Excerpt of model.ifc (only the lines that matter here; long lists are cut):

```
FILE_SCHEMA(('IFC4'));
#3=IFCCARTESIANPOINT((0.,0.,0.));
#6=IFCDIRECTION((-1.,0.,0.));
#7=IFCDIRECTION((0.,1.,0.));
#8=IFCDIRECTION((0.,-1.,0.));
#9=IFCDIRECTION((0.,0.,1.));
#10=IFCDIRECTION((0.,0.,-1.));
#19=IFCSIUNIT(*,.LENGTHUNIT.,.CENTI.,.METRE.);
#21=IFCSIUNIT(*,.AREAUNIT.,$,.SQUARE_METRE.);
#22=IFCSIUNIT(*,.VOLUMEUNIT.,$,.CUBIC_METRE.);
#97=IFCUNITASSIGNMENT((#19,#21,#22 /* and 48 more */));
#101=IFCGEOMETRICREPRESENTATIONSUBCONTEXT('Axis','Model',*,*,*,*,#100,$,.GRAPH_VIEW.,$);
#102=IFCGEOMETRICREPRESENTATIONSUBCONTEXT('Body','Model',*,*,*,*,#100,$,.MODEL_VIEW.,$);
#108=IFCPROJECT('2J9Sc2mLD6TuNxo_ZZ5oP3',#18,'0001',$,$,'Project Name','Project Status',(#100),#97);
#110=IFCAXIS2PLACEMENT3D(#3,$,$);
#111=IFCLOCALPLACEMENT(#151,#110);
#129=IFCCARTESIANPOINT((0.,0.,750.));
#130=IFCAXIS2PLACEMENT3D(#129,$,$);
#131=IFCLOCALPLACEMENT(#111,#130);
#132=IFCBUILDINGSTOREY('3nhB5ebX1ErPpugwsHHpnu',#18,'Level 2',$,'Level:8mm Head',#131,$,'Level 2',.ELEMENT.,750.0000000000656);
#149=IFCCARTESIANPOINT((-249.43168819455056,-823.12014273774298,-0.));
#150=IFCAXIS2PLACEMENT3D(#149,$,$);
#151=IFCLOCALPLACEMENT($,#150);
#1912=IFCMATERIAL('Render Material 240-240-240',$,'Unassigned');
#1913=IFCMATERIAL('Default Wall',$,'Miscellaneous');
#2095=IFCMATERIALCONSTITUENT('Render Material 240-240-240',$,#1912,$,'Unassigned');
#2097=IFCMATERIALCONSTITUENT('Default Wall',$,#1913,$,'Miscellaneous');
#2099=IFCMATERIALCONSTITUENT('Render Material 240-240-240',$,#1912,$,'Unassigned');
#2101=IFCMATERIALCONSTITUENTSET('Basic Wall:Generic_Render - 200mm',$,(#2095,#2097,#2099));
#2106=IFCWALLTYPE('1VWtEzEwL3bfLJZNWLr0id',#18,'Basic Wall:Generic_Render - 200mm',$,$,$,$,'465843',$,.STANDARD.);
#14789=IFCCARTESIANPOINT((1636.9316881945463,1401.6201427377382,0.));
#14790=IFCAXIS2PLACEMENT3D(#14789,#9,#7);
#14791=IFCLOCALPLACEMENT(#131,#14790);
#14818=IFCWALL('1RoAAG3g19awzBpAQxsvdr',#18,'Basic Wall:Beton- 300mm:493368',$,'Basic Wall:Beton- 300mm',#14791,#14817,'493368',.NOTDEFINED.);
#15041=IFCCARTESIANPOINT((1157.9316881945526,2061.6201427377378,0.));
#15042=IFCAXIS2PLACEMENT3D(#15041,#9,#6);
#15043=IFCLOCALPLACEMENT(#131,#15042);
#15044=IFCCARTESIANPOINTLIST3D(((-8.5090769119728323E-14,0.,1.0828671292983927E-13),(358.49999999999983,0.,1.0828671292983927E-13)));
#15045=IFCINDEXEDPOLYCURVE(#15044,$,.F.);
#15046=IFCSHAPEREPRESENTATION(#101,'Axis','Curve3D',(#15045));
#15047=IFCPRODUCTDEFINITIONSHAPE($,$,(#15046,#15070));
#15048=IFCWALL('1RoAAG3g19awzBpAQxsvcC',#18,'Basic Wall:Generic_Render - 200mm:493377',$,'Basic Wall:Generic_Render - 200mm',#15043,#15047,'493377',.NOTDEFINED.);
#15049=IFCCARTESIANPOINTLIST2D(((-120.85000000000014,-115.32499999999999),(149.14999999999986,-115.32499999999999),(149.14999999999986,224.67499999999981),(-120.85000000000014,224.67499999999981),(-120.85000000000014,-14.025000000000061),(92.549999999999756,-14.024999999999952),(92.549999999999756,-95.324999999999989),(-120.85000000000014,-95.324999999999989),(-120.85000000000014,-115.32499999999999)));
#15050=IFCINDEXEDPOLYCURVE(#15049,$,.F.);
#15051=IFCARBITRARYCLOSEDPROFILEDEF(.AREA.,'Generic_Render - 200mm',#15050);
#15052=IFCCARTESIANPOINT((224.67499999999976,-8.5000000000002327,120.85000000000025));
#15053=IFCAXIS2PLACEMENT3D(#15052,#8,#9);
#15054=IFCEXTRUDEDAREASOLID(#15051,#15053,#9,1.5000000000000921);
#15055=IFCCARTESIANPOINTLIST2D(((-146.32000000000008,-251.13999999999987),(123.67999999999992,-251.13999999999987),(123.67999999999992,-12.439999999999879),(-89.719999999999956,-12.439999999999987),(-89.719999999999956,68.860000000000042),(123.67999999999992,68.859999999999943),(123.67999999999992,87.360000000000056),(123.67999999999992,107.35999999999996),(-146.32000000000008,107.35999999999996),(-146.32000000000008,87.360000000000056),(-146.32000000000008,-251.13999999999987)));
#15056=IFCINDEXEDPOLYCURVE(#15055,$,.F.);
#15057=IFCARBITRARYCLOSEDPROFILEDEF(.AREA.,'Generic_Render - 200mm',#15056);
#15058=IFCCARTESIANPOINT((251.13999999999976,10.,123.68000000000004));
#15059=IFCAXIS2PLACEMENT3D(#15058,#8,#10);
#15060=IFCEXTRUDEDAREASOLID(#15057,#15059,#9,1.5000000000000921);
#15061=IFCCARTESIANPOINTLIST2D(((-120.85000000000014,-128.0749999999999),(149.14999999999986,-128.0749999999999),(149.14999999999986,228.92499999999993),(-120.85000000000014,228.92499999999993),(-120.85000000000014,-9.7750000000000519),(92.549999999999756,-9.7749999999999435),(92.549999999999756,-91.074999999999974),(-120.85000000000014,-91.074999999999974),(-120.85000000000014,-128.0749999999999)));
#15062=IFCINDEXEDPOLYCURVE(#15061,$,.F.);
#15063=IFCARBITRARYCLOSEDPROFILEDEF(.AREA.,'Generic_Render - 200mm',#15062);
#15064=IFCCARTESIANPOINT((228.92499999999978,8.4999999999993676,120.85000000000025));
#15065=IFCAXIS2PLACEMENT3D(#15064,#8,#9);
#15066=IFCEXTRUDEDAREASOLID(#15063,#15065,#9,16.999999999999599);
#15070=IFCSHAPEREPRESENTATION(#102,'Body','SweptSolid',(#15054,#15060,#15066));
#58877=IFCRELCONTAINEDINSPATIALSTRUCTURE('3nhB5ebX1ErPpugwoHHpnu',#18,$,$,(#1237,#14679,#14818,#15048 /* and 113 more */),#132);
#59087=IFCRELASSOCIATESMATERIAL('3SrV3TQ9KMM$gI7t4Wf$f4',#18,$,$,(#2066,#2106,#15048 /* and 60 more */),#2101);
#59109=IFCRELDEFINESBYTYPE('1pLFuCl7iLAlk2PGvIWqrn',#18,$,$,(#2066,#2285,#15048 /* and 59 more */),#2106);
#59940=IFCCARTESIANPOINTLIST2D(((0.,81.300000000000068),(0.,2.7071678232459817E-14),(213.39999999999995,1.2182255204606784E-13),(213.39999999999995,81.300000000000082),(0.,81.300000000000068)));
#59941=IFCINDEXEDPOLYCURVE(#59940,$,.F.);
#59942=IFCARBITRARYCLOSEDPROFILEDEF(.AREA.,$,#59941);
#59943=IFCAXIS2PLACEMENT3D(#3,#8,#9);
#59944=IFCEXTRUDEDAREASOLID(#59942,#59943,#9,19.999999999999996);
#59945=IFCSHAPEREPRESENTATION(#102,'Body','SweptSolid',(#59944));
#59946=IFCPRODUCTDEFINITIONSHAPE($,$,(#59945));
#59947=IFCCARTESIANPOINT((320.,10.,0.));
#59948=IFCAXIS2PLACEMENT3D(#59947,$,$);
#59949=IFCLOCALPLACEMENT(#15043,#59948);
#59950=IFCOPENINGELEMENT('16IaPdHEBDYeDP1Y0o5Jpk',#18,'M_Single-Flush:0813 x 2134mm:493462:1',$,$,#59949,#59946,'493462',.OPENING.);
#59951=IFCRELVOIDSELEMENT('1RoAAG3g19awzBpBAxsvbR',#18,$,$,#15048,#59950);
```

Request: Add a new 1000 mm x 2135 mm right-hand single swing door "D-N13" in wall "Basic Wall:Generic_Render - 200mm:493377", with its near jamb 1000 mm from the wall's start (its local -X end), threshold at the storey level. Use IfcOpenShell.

```python
import numpy as np
import ifcopenshell
import ifcopenshell.api.feature
import ifcopenshell.api.geometry
import ifcopenshell.api.root
import ifcopenshell.api.spatial
import ifcopenshell.geom
import ifcopenshell.util.element
import ifcopenshell.util.placement
import ifcopenshell.util.representation
import ifcopenshell.util.shape
import ifcopenshell.util.unit

model = ifcopenshell.open("model.ifc")
unit_scale = ifcopenshell.util.unit.calculate_unit_scale(model)
settings = ifcopenshell.geom.settings()


def volume(element):
    """Net volume in cubic metres, openings subtracted."""
    shape = ifcopenshell.geom.create_shape(settings, element)
    return ifcopenshell.util.shape.get_volume(shape.geometry)


wall = model.by_guid("1RoAAG3g19awzBpAQxsvcC")
storey = ifcopenshell.util.element.get_container(wall, ifc_class="IfcBuildingStorey")
context = ifcopenshell.util.representation.get_context(model, "Model", "Body", "MODEL_VIEW")
before = volume(wall)

width, height, from_end, sill = 1, 2.135, 1, 0.0  # metres

# The wall runs along its own X axis, and the end named is its -X end.
wall_shape = ifcopenshell.geom.create_shape(settings, wall)
x, y, z = ifcopenshell.util.shape.get_vertices(wall_shape.geometry).T
start = x.min() + from_end
face, thickness = float(y.min()), float(y.max() - y.min())
wall_matrix = ifcopenshell.util.placement.get_local_placement(wall.ObjectPlacement)
level = ifcopenshell.util.placement.get_local_placement(storey.ObjectPlacement)[2, 3]


def in_wall(x, y):
    """Placement at x, y metres in the wall's axes, at sill height."""
    matrix = wall_matrix.copy()
    matrix[:, 3] = wall_matrix @ np.array([x / unit_scale, y / unit_scale, 0.0, 1.0])
    matrix[2, 3] = level + sill / unit_scale
    return matrix


# Opening: a box that overshoots both wall faces by 50 mm.
opening = ifcopenshell.api.root.create_entity(model, ifc_class="IfcOpeningElement", predefined_type="OPENING")
box = ifcopenshell.api.geometry.add_wall_representation(
    model, context=context, length=width, height=height, thickness=thickness + 0.1
)
ifcopenshell.api.geometry.assign_representation(model, product=opening, representation=box)
ifcopenshell.api.geometry.edit_object_placement(model, product=opening, matrix=in_wall(start, face - 0.05), is_si=False)
ifcopenshell.api.feature.add_feature(model, feature=opening, element=wall)

door = ifcopenshell.api.root.create_entity(model, ifc_class="IfcDoor", name="D-N13", predefined_type="DOOR")
door.OverallWidth, door.OverallHeight = width / unit_scale, height / unit_scale
door.OperationType = "SINGLE_SWING_RIGHT"
body = ifcopenshell.api.geometry.add_door_representation(
    model,
    context=context,
    overall_width=door.OverallWidth,
    overall_height=door.OverallHeight,
    operation_type="SINGLE_SWING_RIGHT",
    lining_properties={"LiningDepth": thickness / unit_scale, "ThresholdDepth": thickness / unit_scale},
)
ifcopenshell.api.geometry.assign_representation(model, product=door, representation=body)
ifcopenshell.api.spatial.assign_container(model, products=[door], relating_structure=storey)
ifcopenshell.api.feature.add_filling(model, opening=opening, element=door)

# The lining spans the wall, so the door starts at the wall face.
ifcopenshell.api.geometry.edit_object_placement(model, product=door, matrix=in_wall(start, face), is_si=False)

after = volume(wall)

print(f"wall volume {before:.3f} -> {after:.3f} m3")

model.write("model-out.ifc")
```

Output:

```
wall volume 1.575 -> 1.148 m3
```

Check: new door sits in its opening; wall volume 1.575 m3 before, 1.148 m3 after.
